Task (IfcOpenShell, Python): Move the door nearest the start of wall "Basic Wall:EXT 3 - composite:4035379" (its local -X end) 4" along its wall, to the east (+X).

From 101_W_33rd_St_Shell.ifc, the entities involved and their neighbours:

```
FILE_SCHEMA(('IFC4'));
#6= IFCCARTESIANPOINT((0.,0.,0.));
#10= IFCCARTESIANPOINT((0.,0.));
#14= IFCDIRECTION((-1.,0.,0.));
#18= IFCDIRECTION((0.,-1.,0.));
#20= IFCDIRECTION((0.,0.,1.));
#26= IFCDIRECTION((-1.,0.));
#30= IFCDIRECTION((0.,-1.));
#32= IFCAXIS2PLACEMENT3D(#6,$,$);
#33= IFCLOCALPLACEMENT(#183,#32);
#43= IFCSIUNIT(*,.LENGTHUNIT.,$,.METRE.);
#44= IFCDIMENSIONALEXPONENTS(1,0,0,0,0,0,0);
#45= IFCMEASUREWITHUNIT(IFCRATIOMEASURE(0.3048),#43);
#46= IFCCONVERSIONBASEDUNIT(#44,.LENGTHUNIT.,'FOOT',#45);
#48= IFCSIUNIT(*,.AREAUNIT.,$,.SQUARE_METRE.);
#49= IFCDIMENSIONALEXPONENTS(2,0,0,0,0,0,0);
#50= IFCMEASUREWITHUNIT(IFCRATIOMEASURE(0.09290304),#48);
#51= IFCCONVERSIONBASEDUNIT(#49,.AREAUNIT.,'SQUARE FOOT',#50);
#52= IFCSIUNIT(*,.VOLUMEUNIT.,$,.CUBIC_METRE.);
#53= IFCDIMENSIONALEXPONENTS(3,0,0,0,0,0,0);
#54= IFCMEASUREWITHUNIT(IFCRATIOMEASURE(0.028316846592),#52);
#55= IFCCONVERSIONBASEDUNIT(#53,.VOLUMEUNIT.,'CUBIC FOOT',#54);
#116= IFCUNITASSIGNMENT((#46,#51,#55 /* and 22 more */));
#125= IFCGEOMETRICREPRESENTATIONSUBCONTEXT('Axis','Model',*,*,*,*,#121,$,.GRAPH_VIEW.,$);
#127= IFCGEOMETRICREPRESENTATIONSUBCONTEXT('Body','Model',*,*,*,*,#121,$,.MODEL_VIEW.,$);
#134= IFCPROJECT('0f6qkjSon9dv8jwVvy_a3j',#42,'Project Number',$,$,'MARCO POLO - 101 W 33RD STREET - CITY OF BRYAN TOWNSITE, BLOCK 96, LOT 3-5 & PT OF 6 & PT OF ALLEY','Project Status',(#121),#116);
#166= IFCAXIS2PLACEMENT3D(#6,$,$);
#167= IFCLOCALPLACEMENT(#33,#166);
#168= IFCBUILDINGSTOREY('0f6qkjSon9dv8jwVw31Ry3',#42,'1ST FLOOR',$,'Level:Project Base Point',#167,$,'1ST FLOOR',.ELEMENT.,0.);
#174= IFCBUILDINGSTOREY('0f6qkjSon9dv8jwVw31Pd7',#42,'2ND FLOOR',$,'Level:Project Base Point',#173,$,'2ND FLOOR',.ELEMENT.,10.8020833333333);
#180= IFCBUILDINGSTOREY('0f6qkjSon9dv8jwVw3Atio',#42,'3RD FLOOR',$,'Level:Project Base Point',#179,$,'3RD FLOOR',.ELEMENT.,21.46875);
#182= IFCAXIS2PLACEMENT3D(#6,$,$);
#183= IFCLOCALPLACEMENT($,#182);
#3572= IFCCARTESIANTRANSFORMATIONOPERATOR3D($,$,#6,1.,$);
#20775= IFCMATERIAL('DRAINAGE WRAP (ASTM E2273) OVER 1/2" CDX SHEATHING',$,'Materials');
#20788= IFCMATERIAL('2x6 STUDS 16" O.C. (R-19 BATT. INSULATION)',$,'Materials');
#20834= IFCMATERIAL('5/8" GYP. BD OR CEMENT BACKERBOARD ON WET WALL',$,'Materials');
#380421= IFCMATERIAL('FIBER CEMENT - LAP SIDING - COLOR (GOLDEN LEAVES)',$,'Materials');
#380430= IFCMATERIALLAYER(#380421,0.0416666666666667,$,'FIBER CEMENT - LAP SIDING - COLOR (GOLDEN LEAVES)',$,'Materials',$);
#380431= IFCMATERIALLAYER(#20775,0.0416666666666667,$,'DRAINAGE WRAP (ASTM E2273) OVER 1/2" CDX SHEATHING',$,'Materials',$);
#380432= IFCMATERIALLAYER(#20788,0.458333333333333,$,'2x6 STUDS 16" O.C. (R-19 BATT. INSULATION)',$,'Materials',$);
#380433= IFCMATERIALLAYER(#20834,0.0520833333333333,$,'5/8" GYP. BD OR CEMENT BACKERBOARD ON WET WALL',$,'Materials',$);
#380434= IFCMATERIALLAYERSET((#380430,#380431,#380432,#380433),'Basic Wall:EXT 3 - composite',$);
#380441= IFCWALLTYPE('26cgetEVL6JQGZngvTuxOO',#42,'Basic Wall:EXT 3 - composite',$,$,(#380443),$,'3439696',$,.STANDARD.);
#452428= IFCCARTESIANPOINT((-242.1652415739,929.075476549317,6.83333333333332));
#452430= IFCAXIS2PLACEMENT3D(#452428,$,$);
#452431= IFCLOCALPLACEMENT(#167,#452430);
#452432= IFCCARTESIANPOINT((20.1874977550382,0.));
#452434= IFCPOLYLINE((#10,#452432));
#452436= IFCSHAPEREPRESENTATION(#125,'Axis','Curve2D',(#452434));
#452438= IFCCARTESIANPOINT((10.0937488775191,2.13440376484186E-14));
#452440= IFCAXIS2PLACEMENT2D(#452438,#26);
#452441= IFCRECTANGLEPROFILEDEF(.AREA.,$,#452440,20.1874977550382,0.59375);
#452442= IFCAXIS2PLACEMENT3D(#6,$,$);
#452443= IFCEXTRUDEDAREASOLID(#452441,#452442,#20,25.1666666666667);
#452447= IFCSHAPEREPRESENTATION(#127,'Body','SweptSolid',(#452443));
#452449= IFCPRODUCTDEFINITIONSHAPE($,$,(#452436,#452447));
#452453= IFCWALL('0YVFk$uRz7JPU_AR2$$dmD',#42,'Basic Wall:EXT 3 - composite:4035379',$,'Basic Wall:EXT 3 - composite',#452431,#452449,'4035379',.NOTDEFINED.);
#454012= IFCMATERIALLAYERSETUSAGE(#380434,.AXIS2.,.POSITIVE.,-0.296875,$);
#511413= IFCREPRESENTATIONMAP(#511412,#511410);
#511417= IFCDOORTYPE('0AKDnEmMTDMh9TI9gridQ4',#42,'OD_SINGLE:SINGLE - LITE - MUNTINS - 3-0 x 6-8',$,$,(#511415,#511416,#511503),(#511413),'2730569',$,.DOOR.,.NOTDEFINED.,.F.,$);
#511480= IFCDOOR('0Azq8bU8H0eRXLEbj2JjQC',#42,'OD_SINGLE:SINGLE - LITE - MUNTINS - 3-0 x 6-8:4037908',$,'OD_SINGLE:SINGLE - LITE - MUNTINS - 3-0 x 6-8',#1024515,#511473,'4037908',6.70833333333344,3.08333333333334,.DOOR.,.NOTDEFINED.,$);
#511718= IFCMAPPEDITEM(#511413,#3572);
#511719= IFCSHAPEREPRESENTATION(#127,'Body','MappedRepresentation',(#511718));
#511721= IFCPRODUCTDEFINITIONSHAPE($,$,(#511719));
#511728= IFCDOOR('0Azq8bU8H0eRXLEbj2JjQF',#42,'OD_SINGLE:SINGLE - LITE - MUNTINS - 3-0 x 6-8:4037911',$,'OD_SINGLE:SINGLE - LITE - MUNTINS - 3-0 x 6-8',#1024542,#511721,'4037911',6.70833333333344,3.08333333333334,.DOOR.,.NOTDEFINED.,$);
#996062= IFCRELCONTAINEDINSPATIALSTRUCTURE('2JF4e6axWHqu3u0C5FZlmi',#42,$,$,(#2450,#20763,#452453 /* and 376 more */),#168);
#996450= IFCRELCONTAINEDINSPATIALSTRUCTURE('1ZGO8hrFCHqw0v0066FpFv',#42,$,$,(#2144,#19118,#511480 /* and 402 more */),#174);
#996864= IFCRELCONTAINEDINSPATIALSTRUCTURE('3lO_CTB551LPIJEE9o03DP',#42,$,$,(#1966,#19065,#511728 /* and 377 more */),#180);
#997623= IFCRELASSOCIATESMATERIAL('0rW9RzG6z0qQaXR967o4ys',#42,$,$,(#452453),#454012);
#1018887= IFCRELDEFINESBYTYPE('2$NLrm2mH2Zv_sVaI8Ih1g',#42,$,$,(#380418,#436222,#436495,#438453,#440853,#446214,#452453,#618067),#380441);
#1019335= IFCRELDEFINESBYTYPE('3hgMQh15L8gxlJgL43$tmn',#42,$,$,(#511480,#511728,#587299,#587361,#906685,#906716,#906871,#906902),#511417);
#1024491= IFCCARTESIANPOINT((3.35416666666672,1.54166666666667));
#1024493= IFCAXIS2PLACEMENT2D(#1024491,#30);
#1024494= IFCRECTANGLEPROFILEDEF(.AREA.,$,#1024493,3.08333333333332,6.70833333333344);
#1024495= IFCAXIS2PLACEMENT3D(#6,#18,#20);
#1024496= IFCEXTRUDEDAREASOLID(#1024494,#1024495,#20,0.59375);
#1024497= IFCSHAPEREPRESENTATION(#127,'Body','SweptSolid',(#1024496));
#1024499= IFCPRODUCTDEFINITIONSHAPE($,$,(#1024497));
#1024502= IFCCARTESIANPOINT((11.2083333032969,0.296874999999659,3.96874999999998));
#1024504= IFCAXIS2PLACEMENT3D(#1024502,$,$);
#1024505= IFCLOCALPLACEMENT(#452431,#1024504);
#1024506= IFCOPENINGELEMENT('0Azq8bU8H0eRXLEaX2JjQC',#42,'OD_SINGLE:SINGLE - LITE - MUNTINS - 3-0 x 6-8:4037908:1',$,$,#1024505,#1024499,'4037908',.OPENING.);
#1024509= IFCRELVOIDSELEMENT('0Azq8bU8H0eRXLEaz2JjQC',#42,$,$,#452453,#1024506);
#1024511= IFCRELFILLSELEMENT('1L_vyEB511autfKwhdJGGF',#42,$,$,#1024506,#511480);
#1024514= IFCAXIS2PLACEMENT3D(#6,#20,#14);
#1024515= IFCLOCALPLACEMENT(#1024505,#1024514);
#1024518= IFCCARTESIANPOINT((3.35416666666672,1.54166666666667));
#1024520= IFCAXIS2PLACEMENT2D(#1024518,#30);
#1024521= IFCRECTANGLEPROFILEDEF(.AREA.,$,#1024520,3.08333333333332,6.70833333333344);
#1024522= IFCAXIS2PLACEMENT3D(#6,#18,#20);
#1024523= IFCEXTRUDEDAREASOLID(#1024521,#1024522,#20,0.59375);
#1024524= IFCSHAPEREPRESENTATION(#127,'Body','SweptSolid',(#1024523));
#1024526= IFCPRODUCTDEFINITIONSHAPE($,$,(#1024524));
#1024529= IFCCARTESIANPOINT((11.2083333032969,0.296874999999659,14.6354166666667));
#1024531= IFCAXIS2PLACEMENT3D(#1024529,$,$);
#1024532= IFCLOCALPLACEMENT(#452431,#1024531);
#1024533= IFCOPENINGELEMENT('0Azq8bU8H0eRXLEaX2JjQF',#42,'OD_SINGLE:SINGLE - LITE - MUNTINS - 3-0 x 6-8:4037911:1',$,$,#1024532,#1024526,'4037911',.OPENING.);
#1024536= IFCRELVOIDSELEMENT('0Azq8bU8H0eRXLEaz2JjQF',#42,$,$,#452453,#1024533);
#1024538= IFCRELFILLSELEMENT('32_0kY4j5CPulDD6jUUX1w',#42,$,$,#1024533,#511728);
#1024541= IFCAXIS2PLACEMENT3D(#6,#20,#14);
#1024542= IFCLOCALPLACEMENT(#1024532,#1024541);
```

```python
import ifcopenshell
import ifcopenshell.api.geometry
import ifcopenshell.util.placement
import ifcopenshell.util.unit

model = ifcopenshell.open("101_W_33rd_St_Shell.ifc")
unit_scale = ifcopenshell.util.unit.calculate_unit_scale(model)

door = model.by_id(511728)
opening = door.FillsVoids[0].RelatingOpeningElement
wall = opening.VoidsElements[0].RelatingBuildingElement

wall_matrix = ifcopenshell.util.placement.get_local_placement(wall.ObjectPlacement)
shift = wall_matrix[:3, 0] * 4 * 0.0254 / unit_scale
before = ifcopenshell.util.placement.get_local_placement(door.ObjectPlacement)[:3, 3].copy()

# The door is placed relative to its opening, so it follows when the opening moves.
matrix = ifcopenshell.util.placement.get_local_placement(opening.ObjectPlacement)
matrix[:3, 3] += shift
ifcopenshell.api.geometry.edit_object_placement(
    model, product=opening, matrix=matrix, is_si=False, should_transform_children=True
)

after = ifcopenshell.util.placement.get_local_placement(door.ObjectPlacement)[:3, 3]
print("door moved by", (after - before).round(3) + 0.0)

model.write("101_W_33rd_St_Shell_rev.ifc")
```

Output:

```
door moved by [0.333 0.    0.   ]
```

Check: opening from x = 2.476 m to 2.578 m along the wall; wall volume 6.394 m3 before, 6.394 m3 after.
